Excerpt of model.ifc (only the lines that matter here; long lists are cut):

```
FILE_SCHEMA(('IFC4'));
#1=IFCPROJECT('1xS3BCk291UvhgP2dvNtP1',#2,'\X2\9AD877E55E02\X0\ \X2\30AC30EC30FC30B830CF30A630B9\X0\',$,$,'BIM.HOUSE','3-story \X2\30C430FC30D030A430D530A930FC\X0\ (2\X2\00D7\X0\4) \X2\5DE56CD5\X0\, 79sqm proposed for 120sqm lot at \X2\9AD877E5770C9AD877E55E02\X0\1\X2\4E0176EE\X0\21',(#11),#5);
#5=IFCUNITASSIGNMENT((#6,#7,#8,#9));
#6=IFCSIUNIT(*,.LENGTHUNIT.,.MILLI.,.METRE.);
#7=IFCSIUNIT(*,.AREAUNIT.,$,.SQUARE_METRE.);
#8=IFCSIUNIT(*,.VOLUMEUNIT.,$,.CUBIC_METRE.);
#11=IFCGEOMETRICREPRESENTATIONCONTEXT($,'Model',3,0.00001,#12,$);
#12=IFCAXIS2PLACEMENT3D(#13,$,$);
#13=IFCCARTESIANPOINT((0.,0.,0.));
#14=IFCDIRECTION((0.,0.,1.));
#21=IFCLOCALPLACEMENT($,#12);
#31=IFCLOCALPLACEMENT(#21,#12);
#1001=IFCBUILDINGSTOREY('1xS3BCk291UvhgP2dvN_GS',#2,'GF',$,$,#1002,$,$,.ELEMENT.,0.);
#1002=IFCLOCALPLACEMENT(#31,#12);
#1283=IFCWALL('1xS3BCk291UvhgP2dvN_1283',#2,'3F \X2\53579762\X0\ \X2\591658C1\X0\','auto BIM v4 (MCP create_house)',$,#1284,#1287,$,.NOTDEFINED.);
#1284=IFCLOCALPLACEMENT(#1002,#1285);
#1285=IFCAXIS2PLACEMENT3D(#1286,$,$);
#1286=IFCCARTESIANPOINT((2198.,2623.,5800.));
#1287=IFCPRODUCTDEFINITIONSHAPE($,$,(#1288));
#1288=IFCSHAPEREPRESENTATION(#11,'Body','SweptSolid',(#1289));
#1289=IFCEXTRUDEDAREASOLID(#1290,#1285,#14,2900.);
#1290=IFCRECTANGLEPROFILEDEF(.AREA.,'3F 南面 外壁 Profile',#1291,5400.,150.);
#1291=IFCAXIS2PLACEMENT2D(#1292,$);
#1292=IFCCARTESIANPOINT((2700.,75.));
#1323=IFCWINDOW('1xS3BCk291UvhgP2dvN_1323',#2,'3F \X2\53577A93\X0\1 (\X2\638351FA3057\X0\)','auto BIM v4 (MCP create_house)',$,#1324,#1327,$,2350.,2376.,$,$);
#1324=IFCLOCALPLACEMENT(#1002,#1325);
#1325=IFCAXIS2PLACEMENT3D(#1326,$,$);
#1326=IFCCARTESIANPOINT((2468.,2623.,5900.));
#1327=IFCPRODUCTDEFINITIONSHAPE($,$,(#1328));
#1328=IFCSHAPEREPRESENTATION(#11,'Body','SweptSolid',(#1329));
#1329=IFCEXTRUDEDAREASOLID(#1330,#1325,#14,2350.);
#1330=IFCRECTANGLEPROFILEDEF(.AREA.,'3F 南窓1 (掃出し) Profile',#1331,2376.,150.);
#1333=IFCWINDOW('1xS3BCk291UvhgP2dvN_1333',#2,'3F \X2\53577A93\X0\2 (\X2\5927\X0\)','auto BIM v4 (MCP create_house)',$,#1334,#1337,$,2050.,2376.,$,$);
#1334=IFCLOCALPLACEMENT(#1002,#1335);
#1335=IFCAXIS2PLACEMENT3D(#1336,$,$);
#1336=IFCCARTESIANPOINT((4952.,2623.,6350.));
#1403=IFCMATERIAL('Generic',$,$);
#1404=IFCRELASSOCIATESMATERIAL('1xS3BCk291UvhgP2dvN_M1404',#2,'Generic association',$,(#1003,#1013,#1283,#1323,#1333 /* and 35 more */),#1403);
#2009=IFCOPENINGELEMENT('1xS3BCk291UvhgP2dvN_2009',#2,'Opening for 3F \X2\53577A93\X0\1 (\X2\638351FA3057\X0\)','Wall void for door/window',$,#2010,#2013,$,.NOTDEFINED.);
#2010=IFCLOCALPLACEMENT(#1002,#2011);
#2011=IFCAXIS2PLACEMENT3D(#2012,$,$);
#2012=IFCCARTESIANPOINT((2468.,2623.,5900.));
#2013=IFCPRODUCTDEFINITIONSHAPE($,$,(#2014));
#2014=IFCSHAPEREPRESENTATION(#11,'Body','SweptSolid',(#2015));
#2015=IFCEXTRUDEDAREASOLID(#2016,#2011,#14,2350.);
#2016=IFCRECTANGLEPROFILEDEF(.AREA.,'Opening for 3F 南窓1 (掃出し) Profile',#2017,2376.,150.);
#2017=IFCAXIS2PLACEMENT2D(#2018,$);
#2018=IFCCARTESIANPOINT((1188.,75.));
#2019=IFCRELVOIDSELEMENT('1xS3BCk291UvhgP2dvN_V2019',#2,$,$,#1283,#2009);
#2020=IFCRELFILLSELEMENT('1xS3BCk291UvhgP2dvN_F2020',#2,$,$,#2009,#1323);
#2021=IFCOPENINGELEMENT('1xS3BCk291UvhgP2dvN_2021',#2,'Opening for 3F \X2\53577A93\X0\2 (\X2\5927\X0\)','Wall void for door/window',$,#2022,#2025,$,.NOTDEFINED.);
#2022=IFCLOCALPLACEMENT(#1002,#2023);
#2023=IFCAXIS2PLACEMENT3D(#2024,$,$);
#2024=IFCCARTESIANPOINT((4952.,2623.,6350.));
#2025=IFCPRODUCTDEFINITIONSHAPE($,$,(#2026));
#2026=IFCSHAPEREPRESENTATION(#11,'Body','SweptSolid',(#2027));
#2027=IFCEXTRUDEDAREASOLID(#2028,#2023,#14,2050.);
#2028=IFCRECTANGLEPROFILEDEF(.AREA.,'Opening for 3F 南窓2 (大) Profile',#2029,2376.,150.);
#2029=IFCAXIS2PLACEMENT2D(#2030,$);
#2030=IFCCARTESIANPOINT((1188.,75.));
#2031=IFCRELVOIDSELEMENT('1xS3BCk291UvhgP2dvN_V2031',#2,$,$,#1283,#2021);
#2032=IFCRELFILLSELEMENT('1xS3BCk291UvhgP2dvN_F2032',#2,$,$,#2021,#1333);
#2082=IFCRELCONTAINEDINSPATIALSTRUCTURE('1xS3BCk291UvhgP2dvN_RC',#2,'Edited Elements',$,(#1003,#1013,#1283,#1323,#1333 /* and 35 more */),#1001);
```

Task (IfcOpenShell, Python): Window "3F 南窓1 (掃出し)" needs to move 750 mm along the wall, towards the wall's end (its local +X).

```python
import ifcopenshell
import ifcopenshell.api.geometry
import ifcopenshell.util.placement
import ifcopenshell.util.unit

model = ifcopenshell.open("model.ifc")
unit_scale = ifcopenshell.util.unit.calculate_unit_scale(model)

window = model.by_guid("1xS3BCk291UvhgP2dvN_1323")
opening = window.FillsVoids[0].RelatingOpeningElement
wall = opening.VoidsElements[0].RelatingBuildingElement

wall_matrix = ifcopenshell.util.placement.get_local_placement(wall.ObjectPlacement)
shift = wall_matrix[:3, 0] * 0.75 / unit_scale
before = ifcopenshell.util.placement.get_local_placement(window.ObjectPlacement)[:3, 3].copy()

# The window is not placed relative to its opening, so move both.
for product in (opening, window):
    matrix = ifcopenshell.util.placement.get_local_placement(product.ObjectPlacement)
    matrix[:3, 3] += shift
    ifcopenshell.api.geometry.edit_object_placement(model, product=product, matrix=matrix, is_si=False)

after = ifcopenshell.util.placement.get_local_placement(window.ObjectPlacement)[:3, 3]
print("window moved by", (after - before).round(3) + 0.0)

model.write("model_v2.ifc")
```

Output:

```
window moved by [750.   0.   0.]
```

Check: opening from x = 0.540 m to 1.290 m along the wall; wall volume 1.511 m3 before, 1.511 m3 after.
